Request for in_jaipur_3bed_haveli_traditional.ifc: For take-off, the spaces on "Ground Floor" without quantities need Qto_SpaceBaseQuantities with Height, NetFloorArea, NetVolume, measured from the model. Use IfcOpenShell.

First a look at what the model holds.

```python
import ifcopenshell
import ifcopenshell.util.element
import ifcopenshell.util.unit

model = ifcopenshell.open("in_jaipur_3bed_haveli_traditional.ifc")
print(model.schema)
for unit_type in ("LENGTHUNIT", "AREAUNIT", "VOLUMEUNIT"):
    print(unit_type, ifcopenshell.util.unit.calculate_unit_scale(model, unit_type))
storey = next(s for s in model.by_type("IfcBuildingStorey") if s.Name == "Ground Floor")
spaces = [e for e in ifcopenshell.util.element.get_decomposition(storey) if e.is_a("IfcSpace")]
for e in sorted(spaces, key=lambda e: e.id()):
    print(e.id(), e.is_a(), e.Name, list(ifcopenshell.util.element.get_psets(e, qtos_only=True)), sep=" | ")
```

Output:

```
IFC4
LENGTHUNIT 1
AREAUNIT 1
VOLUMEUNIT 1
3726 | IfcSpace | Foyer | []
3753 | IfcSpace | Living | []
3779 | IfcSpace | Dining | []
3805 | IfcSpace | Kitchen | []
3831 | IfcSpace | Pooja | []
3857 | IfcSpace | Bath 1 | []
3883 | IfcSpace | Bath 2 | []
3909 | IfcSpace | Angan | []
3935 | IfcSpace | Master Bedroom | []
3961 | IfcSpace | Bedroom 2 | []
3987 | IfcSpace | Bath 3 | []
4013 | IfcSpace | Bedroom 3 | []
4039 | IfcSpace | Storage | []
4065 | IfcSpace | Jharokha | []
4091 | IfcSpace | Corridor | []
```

```python
import ifcopenshell
import ifcopenshell.api.pset
import ifcopenshell.geom
import ifcopenshell.util.element
import ifcopenshell.util.shape
import ifcopenshell.util.unit

model = ifcopenshell.open("in_jaipur_3bed_haveli_traditional.ifc")
unit_scale = ifcopenshell.util.unit.calculate_unit_scale(model)
area_scale = ifcopenshell.util.unit.calculate_unit_scale(model, "AREAUNIT")
volume_scale = ifcopenshell.util.unit.calculate_unit_scale(model, "VOLUMEUNIT")
settings = ifcopenshell.geom.settings()

storey = next(s for s in model.by_type("IfcBuildingStorey") if s.Name == "Ground Floor")
spaces = [e for e in ifcopenshell.util.element.get_decomposition(storey) if e.is_a("IfcSpace")]

for e in sorted(spaces, key=lambda e: e.id()):
    if ifcopenshell.util.element.get_psets(e, qtos_only=True, should_inherit=False):
        continue
    # Geometry comes back in metres, in the element's own axes.
    shape = ifcopenshell.geom.create_shape(settings, e)
    values = {
        "Height": ifcopenshell.util.shape.get_z(shape.geometry) / unit_scale,
        "NetFloorArea": ifcopenshell.util.shape.get_footprint_area(shape.geometry) / area_scale,
        "NetVolume": ifcopenshell.util.shape.get_volume(shape.geometry) / volume_scale,
    }
    qto = ifcopenshell.api.pset.add_qto(model, product=e, name="Qto_SpaceBaseQuantities")
    ifcopenshell.api.pset.edit_qto(model, qto=qto, properties=values)
    print(e.id(), {k: round(v, 3) for k, v in values.items()})

model.write("in_jaipur_3bed_haveli_traditional_edited.ifc")
```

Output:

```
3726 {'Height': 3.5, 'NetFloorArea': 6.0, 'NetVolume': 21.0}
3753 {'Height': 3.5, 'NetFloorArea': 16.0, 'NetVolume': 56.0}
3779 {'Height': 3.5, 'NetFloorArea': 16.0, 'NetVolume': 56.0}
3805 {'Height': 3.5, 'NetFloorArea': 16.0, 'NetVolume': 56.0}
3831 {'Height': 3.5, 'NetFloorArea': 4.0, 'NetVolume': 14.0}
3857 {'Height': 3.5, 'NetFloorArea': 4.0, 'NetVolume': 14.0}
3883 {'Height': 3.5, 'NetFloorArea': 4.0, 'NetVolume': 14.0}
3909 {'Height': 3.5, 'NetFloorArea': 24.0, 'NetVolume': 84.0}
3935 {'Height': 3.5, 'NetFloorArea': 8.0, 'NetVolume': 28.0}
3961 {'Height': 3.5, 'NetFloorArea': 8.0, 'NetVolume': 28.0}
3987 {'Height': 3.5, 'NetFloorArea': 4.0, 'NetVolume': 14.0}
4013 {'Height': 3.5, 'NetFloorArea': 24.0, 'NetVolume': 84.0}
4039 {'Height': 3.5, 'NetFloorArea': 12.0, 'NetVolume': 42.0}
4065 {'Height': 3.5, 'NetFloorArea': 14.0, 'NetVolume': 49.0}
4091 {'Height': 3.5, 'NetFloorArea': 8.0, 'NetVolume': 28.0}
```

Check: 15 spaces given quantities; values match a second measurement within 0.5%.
